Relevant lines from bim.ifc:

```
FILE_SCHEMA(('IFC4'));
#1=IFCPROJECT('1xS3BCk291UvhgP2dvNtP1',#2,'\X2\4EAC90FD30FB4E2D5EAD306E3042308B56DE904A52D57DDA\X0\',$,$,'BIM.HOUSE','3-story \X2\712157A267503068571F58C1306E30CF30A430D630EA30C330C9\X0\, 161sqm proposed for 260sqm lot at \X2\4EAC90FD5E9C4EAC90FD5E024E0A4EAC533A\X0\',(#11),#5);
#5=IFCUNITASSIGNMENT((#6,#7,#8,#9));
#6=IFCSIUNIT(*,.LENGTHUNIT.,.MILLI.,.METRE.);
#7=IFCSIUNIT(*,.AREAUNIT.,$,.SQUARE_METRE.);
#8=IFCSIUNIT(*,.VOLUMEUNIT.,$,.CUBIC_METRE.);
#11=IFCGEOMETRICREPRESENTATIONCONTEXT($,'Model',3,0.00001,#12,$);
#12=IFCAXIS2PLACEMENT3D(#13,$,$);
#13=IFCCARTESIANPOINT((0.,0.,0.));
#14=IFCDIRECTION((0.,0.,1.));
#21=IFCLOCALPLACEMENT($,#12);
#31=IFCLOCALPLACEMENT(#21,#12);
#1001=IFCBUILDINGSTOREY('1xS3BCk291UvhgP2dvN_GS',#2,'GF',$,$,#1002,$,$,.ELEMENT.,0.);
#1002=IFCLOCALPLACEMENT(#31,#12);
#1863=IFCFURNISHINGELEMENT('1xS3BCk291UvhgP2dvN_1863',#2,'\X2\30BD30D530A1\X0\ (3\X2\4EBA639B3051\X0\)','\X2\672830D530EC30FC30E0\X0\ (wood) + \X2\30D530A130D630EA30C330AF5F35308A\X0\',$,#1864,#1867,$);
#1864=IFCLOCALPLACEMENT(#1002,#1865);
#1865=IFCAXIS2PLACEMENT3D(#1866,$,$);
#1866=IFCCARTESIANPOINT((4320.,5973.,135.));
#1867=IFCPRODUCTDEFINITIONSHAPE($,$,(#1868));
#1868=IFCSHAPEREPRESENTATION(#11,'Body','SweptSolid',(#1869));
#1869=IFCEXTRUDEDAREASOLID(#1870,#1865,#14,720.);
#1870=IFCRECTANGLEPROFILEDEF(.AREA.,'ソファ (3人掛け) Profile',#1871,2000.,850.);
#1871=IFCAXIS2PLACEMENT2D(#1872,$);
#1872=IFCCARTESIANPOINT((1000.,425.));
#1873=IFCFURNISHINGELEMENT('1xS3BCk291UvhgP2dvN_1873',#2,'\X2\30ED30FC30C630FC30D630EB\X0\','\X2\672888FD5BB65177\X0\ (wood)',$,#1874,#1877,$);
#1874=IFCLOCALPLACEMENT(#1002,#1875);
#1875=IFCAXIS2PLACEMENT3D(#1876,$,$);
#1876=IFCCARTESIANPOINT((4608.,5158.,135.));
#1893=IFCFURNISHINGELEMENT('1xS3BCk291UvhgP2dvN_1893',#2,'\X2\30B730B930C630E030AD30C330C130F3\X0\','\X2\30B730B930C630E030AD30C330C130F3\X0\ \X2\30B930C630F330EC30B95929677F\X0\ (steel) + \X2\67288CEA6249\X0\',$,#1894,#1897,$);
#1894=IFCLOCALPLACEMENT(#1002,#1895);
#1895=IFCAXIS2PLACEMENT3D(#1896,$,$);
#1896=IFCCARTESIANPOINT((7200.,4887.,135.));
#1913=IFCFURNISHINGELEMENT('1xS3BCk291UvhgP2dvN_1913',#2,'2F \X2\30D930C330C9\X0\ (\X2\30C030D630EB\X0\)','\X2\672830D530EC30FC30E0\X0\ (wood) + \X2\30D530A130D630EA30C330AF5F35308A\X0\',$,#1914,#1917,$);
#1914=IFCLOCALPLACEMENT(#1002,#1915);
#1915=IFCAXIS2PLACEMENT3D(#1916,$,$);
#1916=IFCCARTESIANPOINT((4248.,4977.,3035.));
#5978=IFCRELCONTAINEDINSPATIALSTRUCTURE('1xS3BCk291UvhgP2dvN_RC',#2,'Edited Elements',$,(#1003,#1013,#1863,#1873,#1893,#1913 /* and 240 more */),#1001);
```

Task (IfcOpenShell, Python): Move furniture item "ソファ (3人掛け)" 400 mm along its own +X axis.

```python
import ifcopenshell
import ifcopenshell.api.geometry
import ifcopenshell.util.placement

model = ifcopenshell.open("bim.ifc")

item = model.by_id(1863)
matrix = ifcopenshell.util.placement.get_local_placement(item.ObjectPlacement)
matrix[:3, 3] += matrix[:3, 0] * 400.0
ifcopenshell.api.geometry.edit_object_placement(model, product=item, matrix=matrix, is_si=False)

print(ifcopenshell.util.placement.get_local_placement(item.ObjectPlacement).round(3) + 0.0)

model.write("bim_rev.ifc")
```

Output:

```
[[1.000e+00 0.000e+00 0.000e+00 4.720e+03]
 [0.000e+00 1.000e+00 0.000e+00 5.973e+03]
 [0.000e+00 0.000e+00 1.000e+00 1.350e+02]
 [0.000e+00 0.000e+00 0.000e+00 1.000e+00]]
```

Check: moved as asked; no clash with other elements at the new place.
